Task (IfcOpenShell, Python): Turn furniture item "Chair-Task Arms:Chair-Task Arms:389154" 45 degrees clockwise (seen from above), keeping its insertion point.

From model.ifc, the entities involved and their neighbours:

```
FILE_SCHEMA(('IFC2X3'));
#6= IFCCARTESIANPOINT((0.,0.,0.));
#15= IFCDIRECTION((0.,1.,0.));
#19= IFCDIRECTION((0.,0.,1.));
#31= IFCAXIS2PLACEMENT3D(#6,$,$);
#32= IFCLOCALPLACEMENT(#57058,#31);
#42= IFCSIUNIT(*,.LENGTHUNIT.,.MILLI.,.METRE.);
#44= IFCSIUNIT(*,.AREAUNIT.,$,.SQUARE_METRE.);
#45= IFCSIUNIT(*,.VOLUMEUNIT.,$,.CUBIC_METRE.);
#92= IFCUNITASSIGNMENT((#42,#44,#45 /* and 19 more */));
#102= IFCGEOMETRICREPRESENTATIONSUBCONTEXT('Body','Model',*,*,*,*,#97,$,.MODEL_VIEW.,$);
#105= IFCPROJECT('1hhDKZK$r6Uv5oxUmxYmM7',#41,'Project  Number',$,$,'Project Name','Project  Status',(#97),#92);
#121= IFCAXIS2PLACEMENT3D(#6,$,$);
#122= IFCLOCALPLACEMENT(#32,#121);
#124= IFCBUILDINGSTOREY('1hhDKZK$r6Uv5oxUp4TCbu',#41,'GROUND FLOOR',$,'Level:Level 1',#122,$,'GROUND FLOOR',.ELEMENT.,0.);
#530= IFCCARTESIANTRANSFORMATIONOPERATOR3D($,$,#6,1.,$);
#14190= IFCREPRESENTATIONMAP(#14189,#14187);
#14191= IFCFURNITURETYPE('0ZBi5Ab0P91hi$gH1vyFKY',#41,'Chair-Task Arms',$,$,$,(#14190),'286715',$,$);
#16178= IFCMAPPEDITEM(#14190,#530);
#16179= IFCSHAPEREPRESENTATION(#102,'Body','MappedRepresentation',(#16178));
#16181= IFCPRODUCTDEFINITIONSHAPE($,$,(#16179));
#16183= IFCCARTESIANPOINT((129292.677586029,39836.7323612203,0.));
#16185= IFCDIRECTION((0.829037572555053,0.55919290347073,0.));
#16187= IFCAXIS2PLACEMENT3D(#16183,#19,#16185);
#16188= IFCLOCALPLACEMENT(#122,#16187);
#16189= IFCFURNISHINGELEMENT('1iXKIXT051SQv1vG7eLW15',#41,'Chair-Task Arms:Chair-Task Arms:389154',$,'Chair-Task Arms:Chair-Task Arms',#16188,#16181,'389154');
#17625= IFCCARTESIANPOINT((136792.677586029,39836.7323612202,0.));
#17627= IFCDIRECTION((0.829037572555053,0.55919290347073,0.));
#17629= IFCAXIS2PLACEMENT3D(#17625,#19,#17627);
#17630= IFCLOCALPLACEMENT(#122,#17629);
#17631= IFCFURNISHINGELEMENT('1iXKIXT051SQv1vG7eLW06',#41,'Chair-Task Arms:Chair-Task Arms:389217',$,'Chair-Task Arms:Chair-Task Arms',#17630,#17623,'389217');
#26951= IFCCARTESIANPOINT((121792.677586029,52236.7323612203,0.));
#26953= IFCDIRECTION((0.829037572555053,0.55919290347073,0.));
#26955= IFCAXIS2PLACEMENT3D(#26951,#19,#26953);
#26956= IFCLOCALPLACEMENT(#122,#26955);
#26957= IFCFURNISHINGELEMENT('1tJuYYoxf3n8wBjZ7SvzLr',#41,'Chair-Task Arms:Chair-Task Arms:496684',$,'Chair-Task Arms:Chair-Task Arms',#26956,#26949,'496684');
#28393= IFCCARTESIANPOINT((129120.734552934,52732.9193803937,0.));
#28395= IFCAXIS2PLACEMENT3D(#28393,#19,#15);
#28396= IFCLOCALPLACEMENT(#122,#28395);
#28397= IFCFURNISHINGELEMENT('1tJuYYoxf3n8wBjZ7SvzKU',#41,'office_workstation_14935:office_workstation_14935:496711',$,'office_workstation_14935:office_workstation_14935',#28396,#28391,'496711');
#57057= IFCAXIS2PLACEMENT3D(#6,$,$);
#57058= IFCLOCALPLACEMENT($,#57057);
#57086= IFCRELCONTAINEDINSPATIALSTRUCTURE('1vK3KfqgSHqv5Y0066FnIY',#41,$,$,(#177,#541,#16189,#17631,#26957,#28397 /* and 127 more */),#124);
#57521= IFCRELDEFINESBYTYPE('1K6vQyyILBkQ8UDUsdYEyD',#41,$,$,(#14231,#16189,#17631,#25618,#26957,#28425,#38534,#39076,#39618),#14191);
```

```python
import ifcopenshell
import ifcopenshell.api.geometry
import ifcopenshell.util.placement

model = ifcopenshell.open("model.ifc")

item = model.by_id(16189)
matrix = ifcopenshell.util.placement.get_local_placement(item.ObjectPlacement)
matrix = matrix @ ifcopenshell.util.placement.rotation(-45, "Z")
ifcopenshell.api.geometry.edit_object_placement(model, product=item, matrix=matrix, is_si=False)

print(ifcopenshell.util.placement.get_local_placement(item.ObjectPlacement).round(3) + 0.0)

model.write("model_v2.ifc")
```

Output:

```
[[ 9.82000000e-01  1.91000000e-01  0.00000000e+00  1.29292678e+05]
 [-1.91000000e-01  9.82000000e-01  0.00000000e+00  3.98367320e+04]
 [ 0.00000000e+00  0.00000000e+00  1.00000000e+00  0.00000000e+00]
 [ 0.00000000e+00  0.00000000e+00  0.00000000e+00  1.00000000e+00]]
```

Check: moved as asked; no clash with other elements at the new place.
